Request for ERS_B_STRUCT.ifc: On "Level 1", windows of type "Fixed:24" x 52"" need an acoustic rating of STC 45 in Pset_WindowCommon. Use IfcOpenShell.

First a look at what the model holds.

```python
import ifcopenshell
import ifcopenshell.util.element

model = ifcopenshell.open("ERS_B_STRUCT.ifc")
print(model.schema)
storey = next(s for s in model.by_type("IfcBuildingStorey") if s.Name == "Level 1")
windows = [e for e in ifcopenshell.util.element.get_decomposition(storey) if e.is_a("IfcWindow")]
seen = {}
for e in windows:
    element_type = ifcopenshell.util.element.get_type(e)
    key = (element_type.Name if element_type != e and element_type else None, ifcopenshell.util.element.get_pset(e, "Pset_WindowCommon", "AcousticRating"))
    seen[key] = seen.get(key, 0) + 1
for (name, value), count in sorted(seen.items(), key=str):
    print(count, "x", name, "|", value)
```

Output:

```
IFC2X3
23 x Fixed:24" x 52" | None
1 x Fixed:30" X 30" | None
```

```python
import ifcopenshell
import ifcopenshell.api.pset
import ifcopenshell.util.element

model = ifcopenshell.open("ERS_B_STRUCT.ifc")

storey = next(s for s in model.by_type("IfcBuildingStorey") if s.Name == "Level 1")
windows = [e for e in ifcopenshell.util.element.get_decomposition(storey) if e.is_a("IfcWindow")]

count = 0
for e in windows:
    element_type = ifcopenshell.util.element.get_type(e)
    if element_type in (None, e) or element_type.Name != 'Fixed:24" x 52"':
        continue
    # add_pset returns the element's existing set when there is one.
    pset = ifcopenshell.api.pset.add_pset(model, product=e, name="Pset_WindowCommon")
    ifcopenshell.api.pset.edit_pset(model, pset=pset, properties={"AcousticRating": "STC 45"})
    count += 1

print(count, "windows updated")

model.write("ERS_B_STRUCT_edited.ifc")
```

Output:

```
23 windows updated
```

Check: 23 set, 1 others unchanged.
